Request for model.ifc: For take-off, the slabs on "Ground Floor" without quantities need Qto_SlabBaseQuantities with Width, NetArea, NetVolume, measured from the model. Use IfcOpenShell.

First a look at what the model holds.

```python
import ifcopenshell
import ifcopenshell.util.element
import ifcopenshell.util.unit

model = ifcopenshell.open("model.ifc")
print(model.schema)
for unit_type in ("LENGTHUNIT", "AREAUNIT", "VOLUMEUNIT"):
    print(unit_type, ifcopenshell.util.unit.calculate_unit_scale(model, unit_type))
storey = next(s for s in model.by_type("IfcBuildingStorey") if s.Name == "Ground Floor")
slabs = [e for e in ifcopenshell.util.element.get_decomposition(storey) if e.is_a("IfcSlab")]
for e in sorted(slabs, key=lambda e: e.id()):
    print(e.id(), e.is_a(), e.Name, list(ifcopenshell.util.element.get_psets(e, qtos_only=True)), sep=" | ")
```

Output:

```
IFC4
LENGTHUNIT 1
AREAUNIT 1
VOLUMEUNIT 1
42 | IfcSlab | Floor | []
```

```python
import ifcopenshell
import ifcopenshell.api.pset
import ifcopenshell.geom
import ifcopenshell.util.element
import ifcopenshell.util.shape
import ifcopenshell.util.unit

model = ifcopenshell.open("model.ifc")
unit_scale = ifcopenshell.util.unit.calculate_unit_scale(model)
area_scale = ifcopenshell.util.unit.calculate_unit_scale(model, "AREAUNIT")
volume_scale = ifcopenshell.util.unit.calculate_unit_scale(model, "VOLUMEUNIT")
settings = ifcopenshell.geom.settings()

storey = next(s for s in model.by_type("IfcBuildingStorey") if s.Name == "Ground Floor")
slabs = [e for e in ifcopenshell.util.element.get_decomposition(storey) if e.is_a("IfcSlab")]

for e in sorted(slabs, key=lambda e: e.id()):
    if ifcopenshell.util.element.get_psets(e, qtos_only=True, should_inherit=False):
        continue
    # Geometry comes back in metres, in the element's own axes.
    shape = ifcopenshell.geom.create_shape(settings, e)
    values = {
        "Width": ifcopenshell.util.shape.get_z(shape.geometry) / unit_scale,
        "NetArea": ifcopenshell.util.shape.get_footprint_area(shape.geometry) / area_scale,
        "NetVolume": ifcopenshell.util.shape.get_volume(shape.geometry) / volume_scale,
    }
    qto = ifcopenshell.api.pset.add_qto(model, product=e, name="Qto_SlabBaseQuantities")
    ifcopenshell.api.pset.edit_qto(model, qto=qto, properties=values)
    print(e.id(), {k: round(v, 3) for k, v in values.items()})

model.write("model_v2.ifc")
```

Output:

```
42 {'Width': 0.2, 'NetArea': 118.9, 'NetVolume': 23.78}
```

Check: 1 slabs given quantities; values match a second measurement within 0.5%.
